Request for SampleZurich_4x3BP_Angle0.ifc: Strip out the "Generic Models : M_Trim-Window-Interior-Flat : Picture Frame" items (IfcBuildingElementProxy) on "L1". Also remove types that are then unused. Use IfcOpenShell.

First a look at what the model holds.

```python
import ifcopenshell
import ifcopenshell.util.element

model = ifcopenshell.open("SampleZurich_4x3BP_Angle0.ifc")
print(model.schema)
storey = next(s for s in model.by_type("IfcBuildingStorey") if s.Name == "L1")
proxies = [e for e in ifcopenshell.util.element.get_decomposition(storey) if e.is_a("IfcBuildingElementProxy")]
seen = {}
for e in proxies:
    element_type = ifcopenshell.util.element.get_type(e)
    name = element_type.Name if element_type not in (None, e) else None
    seen[name] = seen.get(name, 0) + 1
for name, count in sorted(seen.items(), key=str):
    print(count, "x", name)
```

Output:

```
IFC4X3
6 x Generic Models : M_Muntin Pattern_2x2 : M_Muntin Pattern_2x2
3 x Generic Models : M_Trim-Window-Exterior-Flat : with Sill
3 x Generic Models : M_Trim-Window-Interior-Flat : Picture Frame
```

```python
import ifcopenshell
import ifcopenshell.api.root
import ifcopenshell.util.element

model = ifcopenshell.open("SampleZurich_4x3BP_Angle0.ifc")

storey = next(s for s in model.by_type("IfcBuildingStorey") if s.Name == "L1")
proxies = [e for e in ifcopenshell.util.element.get_decomposition(storey) if e.is_a("IfcBuildingElementProxy")]
targets = [e for e in proxies if (t := ifcopenshell.util.element.get_type(e)) not in (None, e) and t.Name == "Generic Models : M_Trim-Window-Interior-Flat : Picture Frame"]
types = {ifcopenshell.util.element.get_type(e) for e in targets} - {None, *targets}

for e in targets:
    ifcopenshell.api.root.remove_product(model, product=e)
print(len(targets), "removed")

unused = [t for t in types if not ifcopenshell.util.element.get_types(t)]
for t in unused:
    ifcopenshell.api.root.remove_product(model, product=t)
print(len(unused), "unused types removed")

model.write("SampleZurich_4x3BP_Angle0_rev.ifc")
```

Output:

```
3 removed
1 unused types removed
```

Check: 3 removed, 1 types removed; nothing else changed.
